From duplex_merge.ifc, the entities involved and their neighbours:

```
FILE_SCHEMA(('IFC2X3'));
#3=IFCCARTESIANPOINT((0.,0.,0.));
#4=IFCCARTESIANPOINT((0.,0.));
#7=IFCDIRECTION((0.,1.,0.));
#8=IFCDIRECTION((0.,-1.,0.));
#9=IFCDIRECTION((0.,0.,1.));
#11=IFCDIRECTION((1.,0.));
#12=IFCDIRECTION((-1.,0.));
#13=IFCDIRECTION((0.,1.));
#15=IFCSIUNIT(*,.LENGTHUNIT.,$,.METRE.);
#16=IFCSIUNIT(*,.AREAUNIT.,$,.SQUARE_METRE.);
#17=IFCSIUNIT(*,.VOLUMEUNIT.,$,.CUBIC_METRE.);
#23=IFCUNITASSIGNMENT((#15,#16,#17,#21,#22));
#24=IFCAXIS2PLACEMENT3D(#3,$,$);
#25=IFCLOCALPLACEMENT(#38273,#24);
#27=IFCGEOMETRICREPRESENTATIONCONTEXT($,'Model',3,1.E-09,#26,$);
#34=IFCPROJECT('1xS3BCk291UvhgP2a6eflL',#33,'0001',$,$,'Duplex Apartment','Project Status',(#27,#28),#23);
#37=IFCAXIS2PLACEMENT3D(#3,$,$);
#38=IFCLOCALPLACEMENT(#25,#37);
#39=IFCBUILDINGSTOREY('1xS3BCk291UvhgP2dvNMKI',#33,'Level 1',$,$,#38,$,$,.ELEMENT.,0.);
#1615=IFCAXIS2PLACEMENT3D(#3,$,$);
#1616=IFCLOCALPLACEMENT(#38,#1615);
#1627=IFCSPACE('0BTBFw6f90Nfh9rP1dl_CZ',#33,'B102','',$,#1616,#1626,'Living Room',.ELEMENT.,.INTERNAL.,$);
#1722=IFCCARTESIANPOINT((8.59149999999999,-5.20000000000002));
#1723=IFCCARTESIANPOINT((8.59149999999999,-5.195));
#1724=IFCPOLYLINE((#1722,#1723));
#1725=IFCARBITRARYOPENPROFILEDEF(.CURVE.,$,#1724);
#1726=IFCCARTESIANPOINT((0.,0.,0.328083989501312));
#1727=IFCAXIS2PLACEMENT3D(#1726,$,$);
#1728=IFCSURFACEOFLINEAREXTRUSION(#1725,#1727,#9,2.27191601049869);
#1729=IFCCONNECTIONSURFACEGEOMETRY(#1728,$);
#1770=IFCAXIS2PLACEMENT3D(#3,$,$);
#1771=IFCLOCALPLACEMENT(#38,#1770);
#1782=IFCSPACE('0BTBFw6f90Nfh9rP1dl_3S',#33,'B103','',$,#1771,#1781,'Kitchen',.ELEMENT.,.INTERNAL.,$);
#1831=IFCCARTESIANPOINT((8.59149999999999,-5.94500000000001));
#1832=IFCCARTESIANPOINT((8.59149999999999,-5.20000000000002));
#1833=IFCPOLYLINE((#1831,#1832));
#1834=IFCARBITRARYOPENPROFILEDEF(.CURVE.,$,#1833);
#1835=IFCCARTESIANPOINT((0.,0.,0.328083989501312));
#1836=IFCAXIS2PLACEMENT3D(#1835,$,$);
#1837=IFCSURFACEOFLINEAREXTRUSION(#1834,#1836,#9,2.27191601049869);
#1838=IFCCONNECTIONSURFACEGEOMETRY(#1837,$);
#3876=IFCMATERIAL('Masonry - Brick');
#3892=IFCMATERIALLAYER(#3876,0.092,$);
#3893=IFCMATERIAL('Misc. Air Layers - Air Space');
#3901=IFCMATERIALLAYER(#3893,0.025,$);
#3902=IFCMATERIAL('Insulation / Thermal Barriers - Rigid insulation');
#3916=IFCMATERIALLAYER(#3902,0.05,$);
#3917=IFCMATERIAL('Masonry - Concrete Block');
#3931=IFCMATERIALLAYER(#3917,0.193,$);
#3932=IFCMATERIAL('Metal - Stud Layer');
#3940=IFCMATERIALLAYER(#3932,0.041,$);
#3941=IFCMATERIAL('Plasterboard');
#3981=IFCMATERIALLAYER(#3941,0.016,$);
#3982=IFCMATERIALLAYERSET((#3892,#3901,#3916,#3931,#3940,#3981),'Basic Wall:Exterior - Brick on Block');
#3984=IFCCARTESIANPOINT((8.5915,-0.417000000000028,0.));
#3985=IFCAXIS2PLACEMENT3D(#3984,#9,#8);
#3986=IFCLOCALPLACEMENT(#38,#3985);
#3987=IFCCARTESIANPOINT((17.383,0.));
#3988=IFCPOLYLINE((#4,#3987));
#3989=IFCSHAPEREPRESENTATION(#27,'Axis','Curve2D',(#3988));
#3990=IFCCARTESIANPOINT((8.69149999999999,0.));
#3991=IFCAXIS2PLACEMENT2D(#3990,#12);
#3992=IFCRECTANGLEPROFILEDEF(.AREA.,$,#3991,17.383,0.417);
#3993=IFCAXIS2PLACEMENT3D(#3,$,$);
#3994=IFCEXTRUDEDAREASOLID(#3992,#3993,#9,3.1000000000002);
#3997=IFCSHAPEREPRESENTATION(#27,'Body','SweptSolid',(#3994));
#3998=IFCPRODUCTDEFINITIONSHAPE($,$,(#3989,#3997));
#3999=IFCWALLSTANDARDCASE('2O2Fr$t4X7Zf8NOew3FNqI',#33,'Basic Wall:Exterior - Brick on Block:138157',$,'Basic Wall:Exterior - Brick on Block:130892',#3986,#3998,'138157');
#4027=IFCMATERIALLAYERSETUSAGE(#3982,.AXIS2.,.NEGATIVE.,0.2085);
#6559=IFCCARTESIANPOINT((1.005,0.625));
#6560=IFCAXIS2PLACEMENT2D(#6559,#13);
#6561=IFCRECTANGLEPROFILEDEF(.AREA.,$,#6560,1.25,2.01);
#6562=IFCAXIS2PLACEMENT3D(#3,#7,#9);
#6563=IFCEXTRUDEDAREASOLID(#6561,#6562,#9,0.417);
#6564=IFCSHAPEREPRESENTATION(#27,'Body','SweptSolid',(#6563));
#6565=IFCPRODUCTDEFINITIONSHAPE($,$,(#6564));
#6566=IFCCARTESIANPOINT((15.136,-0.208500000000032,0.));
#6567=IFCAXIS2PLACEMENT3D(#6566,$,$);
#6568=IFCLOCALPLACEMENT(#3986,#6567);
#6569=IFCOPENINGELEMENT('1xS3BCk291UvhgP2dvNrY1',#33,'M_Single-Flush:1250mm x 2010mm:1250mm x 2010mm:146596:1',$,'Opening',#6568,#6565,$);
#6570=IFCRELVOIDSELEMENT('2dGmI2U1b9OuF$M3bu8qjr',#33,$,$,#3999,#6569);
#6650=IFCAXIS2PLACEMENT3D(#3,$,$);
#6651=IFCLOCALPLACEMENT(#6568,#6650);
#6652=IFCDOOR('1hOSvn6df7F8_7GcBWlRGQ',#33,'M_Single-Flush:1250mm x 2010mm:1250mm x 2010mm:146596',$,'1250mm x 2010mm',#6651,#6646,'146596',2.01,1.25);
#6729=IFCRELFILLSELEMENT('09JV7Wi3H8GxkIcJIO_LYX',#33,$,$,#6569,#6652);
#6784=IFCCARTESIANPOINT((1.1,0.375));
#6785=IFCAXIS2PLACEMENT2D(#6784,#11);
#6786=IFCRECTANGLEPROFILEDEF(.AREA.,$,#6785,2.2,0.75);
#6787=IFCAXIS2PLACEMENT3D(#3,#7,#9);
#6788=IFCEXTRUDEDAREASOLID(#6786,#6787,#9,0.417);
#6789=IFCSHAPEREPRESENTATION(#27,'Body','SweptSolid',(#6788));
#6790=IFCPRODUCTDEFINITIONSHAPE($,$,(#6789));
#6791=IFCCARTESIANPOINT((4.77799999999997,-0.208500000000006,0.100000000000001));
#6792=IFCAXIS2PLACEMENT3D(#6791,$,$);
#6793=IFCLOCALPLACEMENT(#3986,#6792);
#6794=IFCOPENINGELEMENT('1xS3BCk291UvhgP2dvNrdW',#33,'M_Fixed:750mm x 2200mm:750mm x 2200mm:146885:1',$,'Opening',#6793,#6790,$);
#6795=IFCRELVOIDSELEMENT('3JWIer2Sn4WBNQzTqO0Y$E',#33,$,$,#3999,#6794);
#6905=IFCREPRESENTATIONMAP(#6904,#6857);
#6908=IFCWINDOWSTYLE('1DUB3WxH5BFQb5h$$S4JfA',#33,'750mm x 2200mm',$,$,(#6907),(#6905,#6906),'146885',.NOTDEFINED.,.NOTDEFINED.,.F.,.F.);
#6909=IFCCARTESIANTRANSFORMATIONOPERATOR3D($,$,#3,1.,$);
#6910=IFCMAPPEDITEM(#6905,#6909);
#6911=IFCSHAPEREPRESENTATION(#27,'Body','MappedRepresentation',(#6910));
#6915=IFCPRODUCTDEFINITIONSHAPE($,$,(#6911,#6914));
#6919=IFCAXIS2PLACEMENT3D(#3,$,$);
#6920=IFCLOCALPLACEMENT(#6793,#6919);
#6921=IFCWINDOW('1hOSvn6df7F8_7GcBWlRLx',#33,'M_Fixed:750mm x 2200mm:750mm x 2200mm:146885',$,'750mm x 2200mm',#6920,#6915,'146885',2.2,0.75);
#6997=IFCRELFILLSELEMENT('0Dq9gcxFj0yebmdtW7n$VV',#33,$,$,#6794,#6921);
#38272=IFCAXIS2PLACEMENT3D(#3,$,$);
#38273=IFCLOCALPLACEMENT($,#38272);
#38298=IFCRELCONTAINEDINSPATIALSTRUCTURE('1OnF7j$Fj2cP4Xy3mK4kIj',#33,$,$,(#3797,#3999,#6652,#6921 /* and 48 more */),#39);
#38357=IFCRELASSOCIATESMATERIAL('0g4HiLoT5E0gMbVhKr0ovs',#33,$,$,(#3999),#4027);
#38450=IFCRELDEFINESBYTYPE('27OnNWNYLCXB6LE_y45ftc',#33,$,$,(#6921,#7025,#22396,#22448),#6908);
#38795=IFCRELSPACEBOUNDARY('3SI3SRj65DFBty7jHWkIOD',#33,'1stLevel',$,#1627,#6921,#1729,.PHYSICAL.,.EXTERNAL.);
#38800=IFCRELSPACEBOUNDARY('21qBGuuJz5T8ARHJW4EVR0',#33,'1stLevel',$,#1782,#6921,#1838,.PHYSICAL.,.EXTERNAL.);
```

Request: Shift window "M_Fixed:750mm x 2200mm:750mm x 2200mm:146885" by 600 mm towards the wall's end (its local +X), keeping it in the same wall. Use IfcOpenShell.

```python
import numpy as np
import ifcopenshell
import ifcopenshell.api.geometry
import ifcopenshell.util.placement

model = ifcopenshell.open("duplex_merge.ifc")

window = model.by_guid("1hOSvn6df7F8_7GcBWlRLx")
opening = window.FillsVoids[0].RelatingOpeningElement
wall = opening.VoidsElements[0].RelatingBuildingElement

wall_matrix = ifcopenshell.util.placement.get_local_placement(wall.ObjectPlacement)
shift = wall_matrix[:3, 0] * 0.6
before = ifcopenshell.util.placement.get_local_placement(window.ObjectPlacement)[:3, 3].copy()

# The window is placed relative to its opening, so it follows when the opening moves.
matrix = ifcopenshell.util.placement.get_local_placement(opening.ObjectPlacement)
matrix[:3, 3] += shift
ifcopenshell.api.geometry.edit_object_placement(
    model, product=opening, matrix=matrix, is_si=False, should_transform_children=True
)

# Space boundary surfaces are stored in each space's coordinates; move them too.
for rel in window.ProvidesBoundaries:
    if not rel.ConnectionGeometry:
        continue
    surface = rel.ConnectionGeometry.SurfaceOnRelatingElement
    space_matrix = ifcopenshell.util.placement.get_local_placement(rel.RelatingSpace.ObjectPlacement)
    point = np.array(surface.Position.Location.Coordinates) + space_matrix[:3, :3].T @ shift
    surface.Position = model.createIfcAxis2Placement3D(
        model.createIfcCartesianPoint(point.tolist()), surface.Position.Axis, surface.Position.RefDirection
    )

after = ifcopenshell.util.placement.get_local_placement(window.ObjectPlacement)[:3, 3]
print("window moved by", (after - before).round(3) + 0.0)

model.write("duplex_merge_v2.ifc")
```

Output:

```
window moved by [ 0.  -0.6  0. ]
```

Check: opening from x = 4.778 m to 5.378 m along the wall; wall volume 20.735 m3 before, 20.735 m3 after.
